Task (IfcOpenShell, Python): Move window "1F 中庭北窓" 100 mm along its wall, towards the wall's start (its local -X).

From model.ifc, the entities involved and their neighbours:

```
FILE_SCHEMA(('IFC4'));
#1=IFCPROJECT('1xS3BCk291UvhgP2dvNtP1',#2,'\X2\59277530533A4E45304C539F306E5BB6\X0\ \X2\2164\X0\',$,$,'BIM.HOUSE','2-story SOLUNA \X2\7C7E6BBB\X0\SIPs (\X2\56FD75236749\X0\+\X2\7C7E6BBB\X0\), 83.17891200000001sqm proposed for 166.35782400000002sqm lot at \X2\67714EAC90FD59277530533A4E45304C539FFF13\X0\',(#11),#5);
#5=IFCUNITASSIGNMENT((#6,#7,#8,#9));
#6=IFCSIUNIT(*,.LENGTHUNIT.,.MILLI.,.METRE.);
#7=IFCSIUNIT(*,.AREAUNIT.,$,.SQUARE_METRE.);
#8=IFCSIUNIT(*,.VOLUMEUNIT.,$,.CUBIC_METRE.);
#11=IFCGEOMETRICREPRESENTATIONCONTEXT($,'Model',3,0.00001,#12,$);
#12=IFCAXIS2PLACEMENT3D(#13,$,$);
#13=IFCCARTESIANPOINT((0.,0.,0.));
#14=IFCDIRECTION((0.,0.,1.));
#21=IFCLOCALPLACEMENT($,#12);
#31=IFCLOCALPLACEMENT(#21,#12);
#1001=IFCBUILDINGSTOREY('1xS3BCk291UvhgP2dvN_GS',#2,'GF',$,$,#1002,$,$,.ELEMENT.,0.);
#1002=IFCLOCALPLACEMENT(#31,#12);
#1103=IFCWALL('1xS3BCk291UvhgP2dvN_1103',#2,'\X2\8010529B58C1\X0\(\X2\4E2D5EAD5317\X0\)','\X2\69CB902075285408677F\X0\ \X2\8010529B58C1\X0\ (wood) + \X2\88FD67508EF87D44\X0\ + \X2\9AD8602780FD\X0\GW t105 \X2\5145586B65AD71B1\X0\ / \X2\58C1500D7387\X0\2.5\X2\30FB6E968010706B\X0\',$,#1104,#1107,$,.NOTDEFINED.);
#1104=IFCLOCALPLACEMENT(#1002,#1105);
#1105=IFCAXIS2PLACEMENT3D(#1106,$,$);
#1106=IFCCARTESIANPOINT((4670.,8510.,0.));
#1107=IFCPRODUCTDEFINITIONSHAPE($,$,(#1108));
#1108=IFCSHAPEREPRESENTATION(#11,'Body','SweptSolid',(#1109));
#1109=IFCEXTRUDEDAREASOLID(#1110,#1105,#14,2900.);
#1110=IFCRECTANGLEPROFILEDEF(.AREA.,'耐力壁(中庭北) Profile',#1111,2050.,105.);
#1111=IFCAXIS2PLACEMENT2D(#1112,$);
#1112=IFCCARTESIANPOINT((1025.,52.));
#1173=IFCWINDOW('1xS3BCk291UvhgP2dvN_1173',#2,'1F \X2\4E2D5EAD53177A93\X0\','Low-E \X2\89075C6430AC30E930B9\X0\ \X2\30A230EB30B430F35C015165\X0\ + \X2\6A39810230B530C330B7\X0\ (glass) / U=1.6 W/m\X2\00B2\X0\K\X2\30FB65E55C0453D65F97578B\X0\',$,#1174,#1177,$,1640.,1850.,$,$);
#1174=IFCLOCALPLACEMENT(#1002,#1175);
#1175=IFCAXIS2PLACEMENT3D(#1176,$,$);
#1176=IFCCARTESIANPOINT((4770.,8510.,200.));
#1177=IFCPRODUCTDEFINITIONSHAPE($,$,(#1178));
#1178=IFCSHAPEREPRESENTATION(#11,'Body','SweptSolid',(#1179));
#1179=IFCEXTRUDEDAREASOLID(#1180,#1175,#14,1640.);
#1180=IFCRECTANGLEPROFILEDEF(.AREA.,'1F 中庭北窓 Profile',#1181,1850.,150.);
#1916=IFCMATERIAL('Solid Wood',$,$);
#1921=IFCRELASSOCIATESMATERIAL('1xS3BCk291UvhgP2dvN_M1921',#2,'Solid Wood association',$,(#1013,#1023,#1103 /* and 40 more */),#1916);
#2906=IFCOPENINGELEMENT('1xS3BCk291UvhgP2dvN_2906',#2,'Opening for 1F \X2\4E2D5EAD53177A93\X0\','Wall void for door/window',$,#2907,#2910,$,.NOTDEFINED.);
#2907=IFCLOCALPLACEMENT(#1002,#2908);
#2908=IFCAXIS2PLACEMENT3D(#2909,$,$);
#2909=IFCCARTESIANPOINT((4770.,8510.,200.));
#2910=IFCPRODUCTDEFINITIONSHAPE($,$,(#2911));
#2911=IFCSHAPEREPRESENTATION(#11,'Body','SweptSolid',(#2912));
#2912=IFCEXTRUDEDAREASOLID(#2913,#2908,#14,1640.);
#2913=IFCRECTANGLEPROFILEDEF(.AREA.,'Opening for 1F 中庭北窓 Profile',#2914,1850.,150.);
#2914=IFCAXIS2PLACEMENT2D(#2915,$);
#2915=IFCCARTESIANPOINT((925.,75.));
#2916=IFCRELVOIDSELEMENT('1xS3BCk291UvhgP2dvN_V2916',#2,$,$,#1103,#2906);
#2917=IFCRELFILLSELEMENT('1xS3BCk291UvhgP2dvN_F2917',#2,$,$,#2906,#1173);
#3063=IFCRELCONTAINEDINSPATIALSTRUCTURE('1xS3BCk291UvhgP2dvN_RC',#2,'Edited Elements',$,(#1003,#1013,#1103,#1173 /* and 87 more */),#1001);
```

```python
import ifcopenshell
import ifcopenshell.api.geometry
import ifcopenshell.util.placement
import ifcopenshell.util.unit

model = ifcopenshell.open("model.ifc")
unit_scale = ifcopenshell.util.unit.calculate_unit_scale(model)

window = model.by_id(1173)
opening = window.FillsVoids[0].RelatingOpeningElement
wall = opening.VoidsElements[0].RelatingBuildingElement

wall_matrix = ifcopenshell.util.placement.get_local_placement(wall.ObjectPlacement)
shift = wall_matrix[:3, 0] * -0.1 / unit_scale
before = ifcopenshell.util.placement.get_local_placement(window.ObjectPlacement)[:3, 3].copy()

# The window is not placed relative to its opening, so move both.
for product in (opening, window):
    matrix = ifcopenshell.util.placement.get_local_placement(product.ObjectPlacement)
    matrix[:3, 3] += shift
    ifcopenshell.api.geometry.edit_object_placement(model, product=product, matrix=matrix, is_si=False)

after = ifcopenshell.util.placement.get_local_placement(window.ObjectPlacement)[:3, 3]
print("window moved by", (after - before).round(3) + 0.0)

model.write("model-out.ifc")
```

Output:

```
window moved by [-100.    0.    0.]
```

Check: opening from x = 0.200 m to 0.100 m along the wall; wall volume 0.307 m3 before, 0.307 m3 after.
